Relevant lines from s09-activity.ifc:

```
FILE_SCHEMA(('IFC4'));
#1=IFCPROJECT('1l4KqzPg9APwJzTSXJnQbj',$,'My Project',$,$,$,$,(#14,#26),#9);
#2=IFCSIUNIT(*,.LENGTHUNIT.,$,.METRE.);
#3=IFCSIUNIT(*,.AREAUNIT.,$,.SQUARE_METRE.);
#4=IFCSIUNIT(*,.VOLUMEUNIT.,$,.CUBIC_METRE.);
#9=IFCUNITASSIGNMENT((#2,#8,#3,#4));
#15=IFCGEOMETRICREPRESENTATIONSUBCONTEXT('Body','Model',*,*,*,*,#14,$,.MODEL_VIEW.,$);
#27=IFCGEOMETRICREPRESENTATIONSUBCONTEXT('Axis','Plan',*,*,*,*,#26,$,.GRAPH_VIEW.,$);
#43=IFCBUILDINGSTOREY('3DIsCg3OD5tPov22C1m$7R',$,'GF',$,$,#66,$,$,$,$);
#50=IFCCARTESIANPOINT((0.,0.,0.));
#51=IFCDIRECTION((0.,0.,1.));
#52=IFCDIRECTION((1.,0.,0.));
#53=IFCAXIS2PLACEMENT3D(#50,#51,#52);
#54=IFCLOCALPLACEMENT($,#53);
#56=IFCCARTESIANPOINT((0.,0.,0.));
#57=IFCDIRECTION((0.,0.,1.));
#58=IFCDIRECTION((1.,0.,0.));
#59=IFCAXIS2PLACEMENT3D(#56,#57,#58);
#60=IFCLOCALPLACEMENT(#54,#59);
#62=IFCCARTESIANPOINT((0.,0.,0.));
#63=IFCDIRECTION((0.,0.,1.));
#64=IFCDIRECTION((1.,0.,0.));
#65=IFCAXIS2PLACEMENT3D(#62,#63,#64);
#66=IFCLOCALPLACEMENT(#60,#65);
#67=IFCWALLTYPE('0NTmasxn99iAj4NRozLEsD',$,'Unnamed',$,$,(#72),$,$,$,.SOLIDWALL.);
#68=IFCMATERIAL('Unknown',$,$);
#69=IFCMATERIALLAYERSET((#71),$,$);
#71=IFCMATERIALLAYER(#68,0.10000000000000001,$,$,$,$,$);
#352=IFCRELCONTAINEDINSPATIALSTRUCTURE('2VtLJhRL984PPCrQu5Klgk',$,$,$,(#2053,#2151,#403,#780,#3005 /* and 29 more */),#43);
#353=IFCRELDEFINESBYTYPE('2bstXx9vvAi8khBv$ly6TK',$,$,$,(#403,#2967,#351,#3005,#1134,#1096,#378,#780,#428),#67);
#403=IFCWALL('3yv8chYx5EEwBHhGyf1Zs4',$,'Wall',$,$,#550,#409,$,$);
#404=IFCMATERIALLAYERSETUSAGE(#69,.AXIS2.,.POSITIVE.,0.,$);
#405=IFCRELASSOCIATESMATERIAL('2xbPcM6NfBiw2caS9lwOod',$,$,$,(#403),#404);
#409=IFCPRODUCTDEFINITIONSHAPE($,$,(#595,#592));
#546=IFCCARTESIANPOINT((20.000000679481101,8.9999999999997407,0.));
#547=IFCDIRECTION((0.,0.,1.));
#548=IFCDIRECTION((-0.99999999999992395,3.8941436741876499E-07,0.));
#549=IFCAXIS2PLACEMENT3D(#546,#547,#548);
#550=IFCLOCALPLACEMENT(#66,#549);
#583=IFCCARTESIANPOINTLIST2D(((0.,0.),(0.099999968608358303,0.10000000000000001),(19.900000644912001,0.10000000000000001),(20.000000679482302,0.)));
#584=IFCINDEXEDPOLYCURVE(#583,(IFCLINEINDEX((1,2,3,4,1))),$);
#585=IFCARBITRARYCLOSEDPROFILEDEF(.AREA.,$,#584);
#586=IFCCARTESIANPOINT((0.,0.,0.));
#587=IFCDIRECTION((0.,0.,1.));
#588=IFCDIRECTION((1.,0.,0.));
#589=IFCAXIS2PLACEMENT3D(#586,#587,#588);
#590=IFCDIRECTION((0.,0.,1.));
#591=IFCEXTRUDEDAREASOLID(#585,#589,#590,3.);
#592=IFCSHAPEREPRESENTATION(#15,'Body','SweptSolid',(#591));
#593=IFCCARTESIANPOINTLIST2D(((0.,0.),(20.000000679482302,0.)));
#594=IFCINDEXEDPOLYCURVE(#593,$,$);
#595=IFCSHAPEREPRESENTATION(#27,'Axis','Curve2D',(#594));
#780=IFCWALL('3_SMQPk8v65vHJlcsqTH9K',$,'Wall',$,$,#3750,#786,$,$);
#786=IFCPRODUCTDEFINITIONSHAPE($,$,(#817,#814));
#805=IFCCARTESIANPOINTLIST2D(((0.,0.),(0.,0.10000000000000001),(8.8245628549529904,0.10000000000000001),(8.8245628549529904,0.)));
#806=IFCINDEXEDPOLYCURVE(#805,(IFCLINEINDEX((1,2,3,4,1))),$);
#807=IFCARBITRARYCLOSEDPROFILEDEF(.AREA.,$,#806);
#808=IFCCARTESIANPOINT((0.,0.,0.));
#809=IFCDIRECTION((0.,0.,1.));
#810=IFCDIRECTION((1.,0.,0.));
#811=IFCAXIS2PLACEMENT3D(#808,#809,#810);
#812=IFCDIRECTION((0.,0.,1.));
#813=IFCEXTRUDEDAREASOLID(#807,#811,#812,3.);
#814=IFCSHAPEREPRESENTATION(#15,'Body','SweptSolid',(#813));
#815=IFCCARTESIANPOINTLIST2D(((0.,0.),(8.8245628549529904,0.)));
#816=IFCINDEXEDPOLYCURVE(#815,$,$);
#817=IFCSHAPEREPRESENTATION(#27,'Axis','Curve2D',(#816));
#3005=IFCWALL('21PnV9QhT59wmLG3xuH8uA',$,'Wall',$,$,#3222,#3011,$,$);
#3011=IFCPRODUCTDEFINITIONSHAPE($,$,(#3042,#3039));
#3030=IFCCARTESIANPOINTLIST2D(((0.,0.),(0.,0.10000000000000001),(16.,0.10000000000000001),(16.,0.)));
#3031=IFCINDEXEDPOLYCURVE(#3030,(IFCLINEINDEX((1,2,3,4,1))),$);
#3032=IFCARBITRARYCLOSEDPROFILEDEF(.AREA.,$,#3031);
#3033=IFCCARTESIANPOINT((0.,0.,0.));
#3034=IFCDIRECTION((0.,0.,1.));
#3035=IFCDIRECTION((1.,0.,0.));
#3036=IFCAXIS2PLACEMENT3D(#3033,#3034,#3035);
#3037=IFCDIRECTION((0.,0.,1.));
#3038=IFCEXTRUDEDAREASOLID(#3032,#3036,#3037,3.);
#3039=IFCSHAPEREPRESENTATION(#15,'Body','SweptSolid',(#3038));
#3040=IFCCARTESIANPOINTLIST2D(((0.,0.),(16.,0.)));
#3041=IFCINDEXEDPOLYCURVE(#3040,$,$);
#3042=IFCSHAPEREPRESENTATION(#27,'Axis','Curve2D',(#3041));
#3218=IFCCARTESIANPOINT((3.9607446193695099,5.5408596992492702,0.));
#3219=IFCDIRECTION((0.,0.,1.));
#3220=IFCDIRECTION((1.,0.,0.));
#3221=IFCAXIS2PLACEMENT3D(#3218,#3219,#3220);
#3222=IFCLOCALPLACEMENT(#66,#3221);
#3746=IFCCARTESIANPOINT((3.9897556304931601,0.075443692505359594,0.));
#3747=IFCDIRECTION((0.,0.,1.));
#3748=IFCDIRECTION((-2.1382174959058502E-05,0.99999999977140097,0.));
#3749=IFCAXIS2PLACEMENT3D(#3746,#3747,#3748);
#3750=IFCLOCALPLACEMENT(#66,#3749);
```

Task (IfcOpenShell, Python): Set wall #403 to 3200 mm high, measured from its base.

```python
import ifcopenshell
import ifcopenshell.geom
import ifcopenshell.util.representation
import ifcopenshell.util.shape

model = ifcopenshell.open("s09-activity.ifc")
settings = ifcopenshell.geom.settings()


def volume(element):
    """Net volume in cubic metres, openings subtracted."""
    shape = ifcopenshell.geom.create_shape(settings, element)
    return ifcopenshell.util.shape.get_volume(shape.geometry)


wall = model.by_guid("3yv8chYx5EEwBHhGyf1Zs4")
before = volume(wall)

body = ifcopenshell.util.representation.get_representation(wall, "Model", "Body")
solid = body.Items[0]
old_height = solid.Depth
solid.Depth = 3.2
after = volume(wall)

print(f"height {old_height:g} -> {solid.Depth:g}, volume {before:.3f} -> {after:.3f} m3")

model.write("s09-activity_updated.ifc")
```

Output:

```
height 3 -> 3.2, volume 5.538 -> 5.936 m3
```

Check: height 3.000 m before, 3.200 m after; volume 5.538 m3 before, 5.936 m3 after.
